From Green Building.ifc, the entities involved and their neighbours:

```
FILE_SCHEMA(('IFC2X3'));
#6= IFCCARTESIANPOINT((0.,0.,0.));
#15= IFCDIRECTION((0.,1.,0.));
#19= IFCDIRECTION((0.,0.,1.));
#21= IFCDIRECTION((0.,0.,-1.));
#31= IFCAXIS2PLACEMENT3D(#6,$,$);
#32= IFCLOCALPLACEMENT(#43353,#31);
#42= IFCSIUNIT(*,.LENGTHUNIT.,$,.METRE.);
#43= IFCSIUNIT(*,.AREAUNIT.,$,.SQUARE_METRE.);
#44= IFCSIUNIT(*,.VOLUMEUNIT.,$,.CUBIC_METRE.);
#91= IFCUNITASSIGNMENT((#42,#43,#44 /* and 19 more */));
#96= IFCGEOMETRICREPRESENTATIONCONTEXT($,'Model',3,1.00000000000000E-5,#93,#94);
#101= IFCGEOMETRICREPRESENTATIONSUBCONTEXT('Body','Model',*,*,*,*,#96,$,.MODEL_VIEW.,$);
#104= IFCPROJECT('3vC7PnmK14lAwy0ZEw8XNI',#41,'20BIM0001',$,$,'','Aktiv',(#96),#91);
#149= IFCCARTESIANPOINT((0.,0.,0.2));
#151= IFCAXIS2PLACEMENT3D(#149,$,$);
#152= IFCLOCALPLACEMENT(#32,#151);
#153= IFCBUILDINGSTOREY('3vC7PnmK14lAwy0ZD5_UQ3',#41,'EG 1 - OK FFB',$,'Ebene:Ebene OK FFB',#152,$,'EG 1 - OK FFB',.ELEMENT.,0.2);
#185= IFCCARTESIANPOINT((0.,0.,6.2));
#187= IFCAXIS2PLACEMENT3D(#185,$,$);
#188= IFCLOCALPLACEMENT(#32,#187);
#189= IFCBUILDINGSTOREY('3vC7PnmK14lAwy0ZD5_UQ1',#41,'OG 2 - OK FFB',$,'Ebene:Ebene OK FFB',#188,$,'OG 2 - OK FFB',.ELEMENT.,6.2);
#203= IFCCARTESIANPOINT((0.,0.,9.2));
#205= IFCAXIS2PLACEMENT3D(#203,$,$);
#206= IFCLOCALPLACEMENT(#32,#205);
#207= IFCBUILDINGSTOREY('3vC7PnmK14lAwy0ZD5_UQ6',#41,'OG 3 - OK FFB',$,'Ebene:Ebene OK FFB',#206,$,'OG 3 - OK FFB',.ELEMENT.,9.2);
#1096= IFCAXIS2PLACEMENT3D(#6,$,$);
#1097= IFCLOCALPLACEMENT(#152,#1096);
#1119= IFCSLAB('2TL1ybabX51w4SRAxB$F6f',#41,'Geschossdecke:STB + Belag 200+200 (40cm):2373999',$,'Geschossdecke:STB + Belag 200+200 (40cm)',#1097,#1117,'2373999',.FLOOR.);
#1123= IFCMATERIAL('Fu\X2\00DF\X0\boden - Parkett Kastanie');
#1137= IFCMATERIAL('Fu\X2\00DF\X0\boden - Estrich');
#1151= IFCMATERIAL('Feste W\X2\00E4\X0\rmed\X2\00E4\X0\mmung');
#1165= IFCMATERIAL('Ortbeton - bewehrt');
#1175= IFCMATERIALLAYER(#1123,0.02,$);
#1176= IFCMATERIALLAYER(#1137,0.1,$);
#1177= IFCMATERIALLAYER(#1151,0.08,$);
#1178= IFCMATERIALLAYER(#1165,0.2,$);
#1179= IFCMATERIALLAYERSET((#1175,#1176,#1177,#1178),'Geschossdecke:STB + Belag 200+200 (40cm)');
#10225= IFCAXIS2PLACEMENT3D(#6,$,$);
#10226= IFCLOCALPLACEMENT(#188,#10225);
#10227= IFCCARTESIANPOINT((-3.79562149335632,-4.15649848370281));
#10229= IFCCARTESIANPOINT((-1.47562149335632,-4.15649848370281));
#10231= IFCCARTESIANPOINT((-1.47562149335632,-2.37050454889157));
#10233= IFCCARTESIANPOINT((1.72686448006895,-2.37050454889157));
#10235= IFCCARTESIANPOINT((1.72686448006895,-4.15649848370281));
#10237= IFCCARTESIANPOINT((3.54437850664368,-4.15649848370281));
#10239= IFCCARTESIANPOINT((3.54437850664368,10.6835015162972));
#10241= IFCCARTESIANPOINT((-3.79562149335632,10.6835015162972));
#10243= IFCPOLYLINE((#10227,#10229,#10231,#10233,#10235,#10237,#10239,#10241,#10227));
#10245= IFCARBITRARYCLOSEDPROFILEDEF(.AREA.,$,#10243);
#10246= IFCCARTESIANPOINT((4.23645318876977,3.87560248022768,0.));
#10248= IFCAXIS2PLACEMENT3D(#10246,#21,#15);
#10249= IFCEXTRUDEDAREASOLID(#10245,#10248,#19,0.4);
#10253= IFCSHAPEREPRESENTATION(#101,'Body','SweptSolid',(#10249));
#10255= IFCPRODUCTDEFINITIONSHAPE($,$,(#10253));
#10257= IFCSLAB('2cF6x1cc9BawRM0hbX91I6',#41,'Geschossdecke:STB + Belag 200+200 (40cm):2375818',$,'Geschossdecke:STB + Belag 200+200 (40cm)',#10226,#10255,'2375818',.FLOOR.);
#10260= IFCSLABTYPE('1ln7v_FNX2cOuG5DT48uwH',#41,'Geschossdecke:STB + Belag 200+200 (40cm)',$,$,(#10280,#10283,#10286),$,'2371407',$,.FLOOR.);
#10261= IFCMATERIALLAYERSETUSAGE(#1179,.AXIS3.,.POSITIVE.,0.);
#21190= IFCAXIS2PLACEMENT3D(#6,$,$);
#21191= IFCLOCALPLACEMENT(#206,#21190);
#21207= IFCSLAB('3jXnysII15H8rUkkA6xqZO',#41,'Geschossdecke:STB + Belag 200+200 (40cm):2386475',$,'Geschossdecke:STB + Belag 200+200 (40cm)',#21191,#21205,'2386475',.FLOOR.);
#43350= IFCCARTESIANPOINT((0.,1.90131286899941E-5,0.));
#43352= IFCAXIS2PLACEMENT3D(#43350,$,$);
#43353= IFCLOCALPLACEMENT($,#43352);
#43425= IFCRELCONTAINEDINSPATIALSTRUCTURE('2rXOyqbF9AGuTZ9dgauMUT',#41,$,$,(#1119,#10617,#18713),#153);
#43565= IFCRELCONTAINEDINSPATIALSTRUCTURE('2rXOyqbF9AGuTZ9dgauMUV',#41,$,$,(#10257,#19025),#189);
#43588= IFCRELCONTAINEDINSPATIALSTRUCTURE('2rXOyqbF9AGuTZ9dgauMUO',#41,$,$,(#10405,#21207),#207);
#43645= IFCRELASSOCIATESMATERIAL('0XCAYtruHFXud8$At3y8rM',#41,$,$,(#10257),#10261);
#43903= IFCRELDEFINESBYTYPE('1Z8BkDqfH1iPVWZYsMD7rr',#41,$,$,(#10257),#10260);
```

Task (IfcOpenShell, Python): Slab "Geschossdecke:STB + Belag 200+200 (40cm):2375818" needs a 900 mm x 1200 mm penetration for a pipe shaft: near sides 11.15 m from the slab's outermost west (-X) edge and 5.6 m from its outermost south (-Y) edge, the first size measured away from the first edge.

```python
import numpy as np
import ifcopenshell
import ifcopenshell.api.feature
import ifcopenshell.api.geometry
import ifcopenshell.api.root
import ifcopenshell.geom
import ifcopenshell.util.placement
import ifcopenshell.util.representation
import ifcopenshell.util.shape
import ifcopenshell.util.unit

model = ifcopenshell.open("Green Building.ifc")
unit_scale = ifcopenshell.util.unit.calculate_unit_scale(model)
settings = ifcopenshell.geom.settings()


def volume(element):
    """Net volume in cubic metres, openings subtracted."""
    shape = ifcopenshell.geom.create_shape(settings, element)
    return ifcopenshell.util.shape.get_volume(shape.geometry)


slab = model.by_guid("2cF6x1cc9BawRM0hbX91I6")
before = volume(slab)

# Extent in the slab's own axes, in metres. The edges named are its -X and -Y sides.
slab_shape = ifcopenshell.geom.create_shape(settings, slab)
vertices = ifcopenshell.util.shape.get_vertices(slab_shape.geometry)
x_min, y_min, bottom = vertices.min(axis=0)
top = vertices[:, 2].max()

opening = ifcopenshell.api.root.create_entity(model, ifc_class="IfcOpeningElement", name="Pipe shaft opening")
context = ifcopenshell.util.representation.get_context(model, "Model", "Body", "MODEL_VIEW")
width, depth = 0.9, 1.2
outline = [(0.0, 0.0), (width, 0.0), (width, depth), (0.0, depth), (0.0, 0.0)]
# Overshoot both faces by 50 mm so the cut is clean.
shape = ifcopenshell.api.geometry.add_slab_representation(
    model, context=context, depth=top - bottom + 0.1, polyline=outline
)
ifcopenshell.api.geometry.assign_representation(model, product=opening, representation=shape)

matrix = ifcopenshell.util.placement.get_local_placement(slab.ObjectPlacement)
matrix[:, 3] = matrix @ np.append(np.array([x_min + 11.15, y_min + 5.6, bottom - 0.05]) / unit_scale, 1.0)
ifcopenshell.api.geometry.edit_object_placement(model, product=opening, matrix=matrix, is_si=False)
ifcopenshell.api.feature.add_feature(model, feature=opening, element=slab)

after = volume(slab)

print(f"slab volume {before:.3f} -> {after:.3f} m3")

model.write("Green Building_rev.ifc")
```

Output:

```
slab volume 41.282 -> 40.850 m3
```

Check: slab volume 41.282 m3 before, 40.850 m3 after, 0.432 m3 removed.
